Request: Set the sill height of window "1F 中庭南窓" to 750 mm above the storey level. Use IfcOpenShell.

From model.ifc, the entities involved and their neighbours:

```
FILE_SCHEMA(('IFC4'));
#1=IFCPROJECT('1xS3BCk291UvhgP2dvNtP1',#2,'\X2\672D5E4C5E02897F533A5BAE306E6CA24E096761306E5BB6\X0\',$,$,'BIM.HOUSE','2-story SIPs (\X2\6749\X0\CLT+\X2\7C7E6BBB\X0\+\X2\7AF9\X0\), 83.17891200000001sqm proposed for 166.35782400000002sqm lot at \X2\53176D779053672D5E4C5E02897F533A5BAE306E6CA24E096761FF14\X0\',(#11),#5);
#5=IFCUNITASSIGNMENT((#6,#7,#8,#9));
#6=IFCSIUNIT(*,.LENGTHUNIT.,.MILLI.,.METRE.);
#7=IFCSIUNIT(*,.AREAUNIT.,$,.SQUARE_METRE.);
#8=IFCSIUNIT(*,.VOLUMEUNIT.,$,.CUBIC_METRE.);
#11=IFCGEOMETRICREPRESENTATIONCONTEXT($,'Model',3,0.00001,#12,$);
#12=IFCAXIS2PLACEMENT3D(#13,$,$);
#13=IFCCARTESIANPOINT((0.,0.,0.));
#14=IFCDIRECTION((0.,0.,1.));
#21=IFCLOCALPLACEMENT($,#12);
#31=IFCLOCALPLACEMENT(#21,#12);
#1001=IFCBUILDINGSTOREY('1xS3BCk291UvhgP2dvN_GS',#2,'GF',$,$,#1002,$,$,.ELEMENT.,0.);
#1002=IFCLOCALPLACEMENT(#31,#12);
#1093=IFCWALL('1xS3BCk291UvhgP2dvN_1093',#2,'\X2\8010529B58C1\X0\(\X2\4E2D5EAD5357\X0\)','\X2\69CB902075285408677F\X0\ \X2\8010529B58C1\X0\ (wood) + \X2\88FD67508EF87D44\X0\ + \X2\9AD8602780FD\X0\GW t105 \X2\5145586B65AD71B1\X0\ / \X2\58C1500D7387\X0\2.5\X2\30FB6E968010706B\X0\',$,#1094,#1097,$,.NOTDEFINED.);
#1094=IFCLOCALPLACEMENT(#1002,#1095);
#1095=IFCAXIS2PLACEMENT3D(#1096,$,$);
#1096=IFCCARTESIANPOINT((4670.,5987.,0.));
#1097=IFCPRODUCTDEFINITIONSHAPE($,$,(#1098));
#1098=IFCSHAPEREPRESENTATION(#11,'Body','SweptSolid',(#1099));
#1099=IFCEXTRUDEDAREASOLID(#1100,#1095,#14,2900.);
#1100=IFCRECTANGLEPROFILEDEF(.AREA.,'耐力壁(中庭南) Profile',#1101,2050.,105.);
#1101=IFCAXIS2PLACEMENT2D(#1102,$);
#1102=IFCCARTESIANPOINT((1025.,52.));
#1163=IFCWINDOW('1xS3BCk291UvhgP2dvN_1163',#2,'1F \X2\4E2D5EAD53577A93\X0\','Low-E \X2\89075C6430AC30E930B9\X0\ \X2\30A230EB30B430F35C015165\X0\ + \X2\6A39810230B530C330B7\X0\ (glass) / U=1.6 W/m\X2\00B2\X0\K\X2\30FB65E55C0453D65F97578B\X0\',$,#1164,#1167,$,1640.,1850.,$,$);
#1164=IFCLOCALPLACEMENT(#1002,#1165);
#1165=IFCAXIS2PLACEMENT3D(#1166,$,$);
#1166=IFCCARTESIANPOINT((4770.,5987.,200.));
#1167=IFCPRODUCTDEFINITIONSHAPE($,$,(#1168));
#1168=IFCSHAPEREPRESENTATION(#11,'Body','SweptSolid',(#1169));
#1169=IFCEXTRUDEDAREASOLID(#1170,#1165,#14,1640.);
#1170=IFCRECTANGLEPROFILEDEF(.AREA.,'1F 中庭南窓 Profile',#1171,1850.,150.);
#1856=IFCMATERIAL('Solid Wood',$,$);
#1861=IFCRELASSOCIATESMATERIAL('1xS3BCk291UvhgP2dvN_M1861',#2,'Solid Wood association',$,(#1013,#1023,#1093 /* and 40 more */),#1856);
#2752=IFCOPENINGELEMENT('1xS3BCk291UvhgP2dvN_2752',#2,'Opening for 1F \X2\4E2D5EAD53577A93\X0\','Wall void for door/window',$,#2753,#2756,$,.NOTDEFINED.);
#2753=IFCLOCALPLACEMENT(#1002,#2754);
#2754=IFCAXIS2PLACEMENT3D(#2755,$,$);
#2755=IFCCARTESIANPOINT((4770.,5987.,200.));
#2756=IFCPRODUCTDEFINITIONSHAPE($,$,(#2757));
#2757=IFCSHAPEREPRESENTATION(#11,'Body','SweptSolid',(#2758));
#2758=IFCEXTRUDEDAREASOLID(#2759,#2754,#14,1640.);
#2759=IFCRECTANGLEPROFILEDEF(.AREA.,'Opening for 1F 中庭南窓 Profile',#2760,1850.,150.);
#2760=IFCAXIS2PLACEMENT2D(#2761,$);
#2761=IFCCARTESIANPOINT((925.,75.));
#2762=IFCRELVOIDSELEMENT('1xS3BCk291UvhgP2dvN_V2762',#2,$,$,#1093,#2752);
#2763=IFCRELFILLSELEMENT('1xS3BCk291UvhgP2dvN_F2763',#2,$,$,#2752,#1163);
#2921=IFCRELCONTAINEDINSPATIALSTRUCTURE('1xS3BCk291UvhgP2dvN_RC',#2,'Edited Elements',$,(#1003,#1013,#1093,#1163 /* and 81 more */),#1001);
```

```python
import numpy as np
import ifcopenshell
import ifcopenshell.api.geometry
import ifcopenshell.geom
import ifcopenshell.util.element
import ifcopenshell.util.placement
import ifcopenshell.util.shape
import ifcopenshell.util.unit

model = ifcopenshell.open("model.ifc")
unit_scale = ifcopenshell.util.unit.calculate_unit_scale(model)

window = model.by_guid("1xS3BCk291UvhgP2dvN_1163")
opening = window.FillsVoids[0].RelatingOpeningElement
storey = ifcopenshell.util.element.get_container(window, ifc_class="IfcBuildingStorey")
level = ifcopenshell.util.placement.get_local_placement(storey.ObjectPlacement)[2, 3]

# The opening's origin need not be at the sill, so measure its lowest point.
shape = ifcopenshell.geom.create_shape(ifcopenshell.geom.settings(), opening)
bottom = ifcopenshell.util.shape.get_shape_bottom_elevation(shape, shape.geometry) / unit_scale
dz = level + 0.75 / unit_scale - bottom

shift = np.array([0.0, 0.0, dz])
# The window is not placed relative to its opening, so move both.
for product in (opening, window):
    matrix = ifcopenshell.util.placement.get_local_placement(product.ObjectPlacement)
    matrix[:3, 3] += shift
    ifcopenshell.api.geometry.edit_object_placement(model, product=product, matrix=matrix, is_si=False)

print(f"moved by {dz * unit_scale:+.3f} m")

model.write("model_updated.ifc")
```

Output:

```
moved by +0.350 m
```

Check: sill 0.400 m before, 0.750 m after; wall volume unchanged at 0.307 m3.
